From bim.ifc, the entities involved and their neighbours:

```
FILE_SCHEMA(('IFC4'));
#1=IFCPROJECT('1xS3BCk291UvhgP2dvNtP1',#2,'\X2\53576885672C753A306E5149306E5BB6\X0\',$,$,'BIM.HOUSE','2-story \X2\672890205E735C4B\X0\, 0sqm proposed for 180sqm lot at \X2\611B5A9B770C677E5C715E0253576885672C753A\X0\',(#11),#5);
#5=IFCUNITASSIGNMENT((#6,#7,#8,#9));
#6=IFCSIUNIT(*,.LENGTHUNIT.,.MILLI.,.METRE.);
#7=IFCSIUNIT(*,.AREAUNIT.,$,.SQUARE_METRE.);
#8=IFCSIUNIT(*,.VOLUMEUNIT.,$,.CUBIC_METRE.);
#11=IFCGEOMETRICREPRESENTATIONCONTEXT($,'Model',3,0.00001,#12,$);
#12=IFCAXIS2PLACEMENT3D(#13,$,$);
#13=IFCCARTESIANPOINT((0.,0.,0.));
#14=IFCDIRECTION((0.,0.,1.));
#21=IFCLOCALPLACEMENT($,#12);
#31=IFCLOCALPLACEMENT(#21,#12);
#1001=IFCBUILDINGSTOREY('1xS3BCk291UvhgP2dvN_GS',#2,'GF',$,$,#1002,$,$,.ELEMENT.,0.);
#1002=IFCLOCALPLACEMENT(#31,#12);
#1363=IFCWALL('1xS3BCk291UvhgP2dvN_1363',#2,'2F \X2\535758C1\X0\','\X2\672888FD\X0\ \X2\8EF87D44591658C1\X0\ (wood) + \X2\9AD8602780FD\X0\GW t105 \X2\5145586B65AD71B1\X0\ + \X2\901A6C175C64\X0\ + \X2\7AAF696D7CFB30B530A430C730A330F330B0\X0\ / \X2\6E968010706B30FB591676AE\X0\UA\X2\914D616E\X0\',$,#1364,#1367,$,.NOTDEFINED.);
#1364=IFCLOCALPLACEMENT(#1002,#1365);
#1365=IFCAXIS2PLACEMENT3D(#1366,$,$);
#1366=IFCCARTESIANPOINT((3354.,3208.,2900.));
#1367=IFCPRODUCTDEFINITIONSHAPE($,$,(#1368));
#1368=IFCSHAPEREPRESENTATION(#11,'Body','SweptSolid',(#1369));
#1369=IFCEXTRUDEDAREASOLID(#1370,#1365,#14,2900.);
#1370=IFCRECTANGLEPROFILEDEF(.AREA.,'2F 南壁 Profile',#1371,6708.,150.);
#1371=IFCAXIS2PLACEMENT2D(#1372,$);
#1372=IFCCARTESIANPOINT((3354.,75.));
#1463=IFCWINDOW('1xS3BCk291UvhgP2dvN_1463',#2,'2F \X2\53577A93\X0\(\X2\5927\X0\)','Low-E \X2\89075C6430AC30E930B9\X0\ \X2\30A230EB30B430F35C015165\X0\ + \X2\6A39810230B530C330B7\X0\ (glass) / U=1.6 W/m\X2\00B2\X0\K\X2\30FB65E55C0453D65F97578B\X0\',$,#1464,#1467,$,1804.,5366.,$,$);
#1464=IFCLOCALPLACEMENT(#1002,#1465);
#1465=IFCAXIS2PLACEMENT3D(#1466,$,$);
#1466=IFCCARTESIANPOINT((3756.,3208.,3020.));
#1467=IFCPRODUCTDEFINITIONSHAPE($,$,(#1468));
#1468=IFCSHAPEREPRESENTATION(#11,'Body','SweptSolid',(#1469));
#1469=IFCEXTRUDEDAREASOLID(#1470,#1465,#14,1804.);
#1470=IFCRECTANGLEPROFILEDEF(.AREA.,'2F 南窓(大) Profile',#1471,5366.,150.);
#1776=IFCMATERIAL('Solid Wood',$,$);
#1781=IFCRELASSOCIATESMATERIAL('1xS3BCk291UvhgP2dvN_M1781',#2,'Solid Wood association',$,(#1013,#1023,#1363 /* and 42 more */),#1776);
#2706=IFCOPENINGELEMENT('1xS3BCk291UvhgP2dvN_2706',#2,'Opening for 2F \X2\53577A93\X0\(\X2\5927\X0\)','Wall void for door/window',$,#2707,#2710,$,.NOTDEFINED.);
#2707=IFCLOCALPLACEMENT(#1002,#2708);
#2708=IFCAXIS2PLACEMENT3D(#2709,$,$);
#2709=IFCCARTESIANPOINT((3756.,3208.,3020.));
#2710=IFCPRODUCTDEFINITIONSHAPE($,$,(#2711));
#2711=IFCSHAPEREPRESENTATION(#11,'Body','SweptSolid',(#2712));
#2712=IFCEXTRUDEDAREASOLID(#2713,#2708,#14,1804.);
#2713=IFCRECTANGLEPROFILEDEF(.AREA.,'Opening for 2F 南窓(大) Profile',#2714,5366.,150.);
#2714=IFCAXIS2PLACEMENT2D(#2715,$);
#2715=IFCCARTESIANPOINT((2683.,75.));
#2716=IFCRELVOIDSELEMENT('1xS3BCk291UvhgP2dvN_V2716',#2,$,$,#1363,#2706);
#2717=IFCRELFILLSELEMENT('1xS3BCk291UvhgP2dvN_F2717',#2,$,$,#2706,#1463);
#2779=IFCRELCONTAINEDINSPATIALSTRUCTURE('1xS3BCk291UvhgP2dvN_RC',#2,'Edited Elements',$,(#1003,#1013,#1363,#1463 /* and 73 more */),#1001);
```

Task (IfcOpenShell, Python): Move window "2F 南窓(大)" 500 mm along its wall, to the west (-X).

```python
import ifcopenshell
import ifcopenshell.api.geometry
import ifcopenshell.util.placement
import ifcopenshell.util.unit

model = ifcopenshell.open("bim.ifc")
unit_scale = ifcopenshell.util.unit.calculate_unit_scale(model)

window = model.by_id(1463)
opening = window.FillsVoids[0].RelatingOpeningElement
wall = opening.VoidsElements[0].RelatingBuildingElement

wall_matrix = ifcopenshell.util.placement.get_local_placement(wall.ObjectPlacement)
shift = wall_matrix[:3, 0] * -0.5 / unit_scale
before = ifcopenshell.util.placement.get_local_placement(window.ObjectPlacement)[:3, 3].copy()

# The window is not placed relative to its opening, so move both.
for product in (opening, window):
    matrix = ifcopenshell.util.placement.get_local_placement(product.ObjectPlacement)
    matrix[:3, 3] += shift
    ifcopenshell.api.geometry.edit_object_placement(model, product=product, matrix=matrix, is_si=False)

after = ifcopenshell.util.placement.get_local_placement(window.ObjectPlacement)[:3, 3]
print("window moved by", (after - before).round(3) + 0.0)

model.write("bim_edited.ifc")
```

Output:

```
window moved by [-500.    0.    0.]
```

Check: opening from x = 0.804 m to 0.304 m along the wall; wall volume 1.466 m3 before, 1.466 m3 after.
